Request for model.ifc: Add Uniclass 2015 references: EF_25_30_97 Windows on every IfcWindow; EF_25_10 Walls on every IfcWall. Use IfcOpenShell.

First a look at what the model holds.

```python
import ifcopenshell

model = ifcopenshell.open("model.ifc")
print(model.schema)
print("classifications:", [c.Name for c in model.by_type("IfcClassification")])
for ifc_class in ("IfcDoor", "IfcRoof", "IfcStair", "IfcWall", "IfcWindow"):
    print(ifc_class, len(model.by_type(ifc_class)))
```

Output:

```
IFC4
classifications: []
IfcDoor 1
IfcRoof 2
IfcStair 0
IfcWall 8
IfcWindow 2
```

```python
import ifcopenshell
import ifcopenshell.api.classification

model = ifcopenshell.open("model.ifc")

system = ifcopenshell.api.classification.add_classification(model, classification="Uniclass 2015")

codes = {
    "IfcWindow": ("EF_25_30_97", "Windows"),
    "IfcWall": ("EF_25_10", "Walls"),
}
for ifc_class, (code, name) in codes.items():
    products = model.by_type(ifc_class)
    ifcopenshell.api.classification.add_reference(
        model, products=products, classification=system, identification=code, name=name
    )
    print(code, len(products))

model.write("model_rev.ifc")
```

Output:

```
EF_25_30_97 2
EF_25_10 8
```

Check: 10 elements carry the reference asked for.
